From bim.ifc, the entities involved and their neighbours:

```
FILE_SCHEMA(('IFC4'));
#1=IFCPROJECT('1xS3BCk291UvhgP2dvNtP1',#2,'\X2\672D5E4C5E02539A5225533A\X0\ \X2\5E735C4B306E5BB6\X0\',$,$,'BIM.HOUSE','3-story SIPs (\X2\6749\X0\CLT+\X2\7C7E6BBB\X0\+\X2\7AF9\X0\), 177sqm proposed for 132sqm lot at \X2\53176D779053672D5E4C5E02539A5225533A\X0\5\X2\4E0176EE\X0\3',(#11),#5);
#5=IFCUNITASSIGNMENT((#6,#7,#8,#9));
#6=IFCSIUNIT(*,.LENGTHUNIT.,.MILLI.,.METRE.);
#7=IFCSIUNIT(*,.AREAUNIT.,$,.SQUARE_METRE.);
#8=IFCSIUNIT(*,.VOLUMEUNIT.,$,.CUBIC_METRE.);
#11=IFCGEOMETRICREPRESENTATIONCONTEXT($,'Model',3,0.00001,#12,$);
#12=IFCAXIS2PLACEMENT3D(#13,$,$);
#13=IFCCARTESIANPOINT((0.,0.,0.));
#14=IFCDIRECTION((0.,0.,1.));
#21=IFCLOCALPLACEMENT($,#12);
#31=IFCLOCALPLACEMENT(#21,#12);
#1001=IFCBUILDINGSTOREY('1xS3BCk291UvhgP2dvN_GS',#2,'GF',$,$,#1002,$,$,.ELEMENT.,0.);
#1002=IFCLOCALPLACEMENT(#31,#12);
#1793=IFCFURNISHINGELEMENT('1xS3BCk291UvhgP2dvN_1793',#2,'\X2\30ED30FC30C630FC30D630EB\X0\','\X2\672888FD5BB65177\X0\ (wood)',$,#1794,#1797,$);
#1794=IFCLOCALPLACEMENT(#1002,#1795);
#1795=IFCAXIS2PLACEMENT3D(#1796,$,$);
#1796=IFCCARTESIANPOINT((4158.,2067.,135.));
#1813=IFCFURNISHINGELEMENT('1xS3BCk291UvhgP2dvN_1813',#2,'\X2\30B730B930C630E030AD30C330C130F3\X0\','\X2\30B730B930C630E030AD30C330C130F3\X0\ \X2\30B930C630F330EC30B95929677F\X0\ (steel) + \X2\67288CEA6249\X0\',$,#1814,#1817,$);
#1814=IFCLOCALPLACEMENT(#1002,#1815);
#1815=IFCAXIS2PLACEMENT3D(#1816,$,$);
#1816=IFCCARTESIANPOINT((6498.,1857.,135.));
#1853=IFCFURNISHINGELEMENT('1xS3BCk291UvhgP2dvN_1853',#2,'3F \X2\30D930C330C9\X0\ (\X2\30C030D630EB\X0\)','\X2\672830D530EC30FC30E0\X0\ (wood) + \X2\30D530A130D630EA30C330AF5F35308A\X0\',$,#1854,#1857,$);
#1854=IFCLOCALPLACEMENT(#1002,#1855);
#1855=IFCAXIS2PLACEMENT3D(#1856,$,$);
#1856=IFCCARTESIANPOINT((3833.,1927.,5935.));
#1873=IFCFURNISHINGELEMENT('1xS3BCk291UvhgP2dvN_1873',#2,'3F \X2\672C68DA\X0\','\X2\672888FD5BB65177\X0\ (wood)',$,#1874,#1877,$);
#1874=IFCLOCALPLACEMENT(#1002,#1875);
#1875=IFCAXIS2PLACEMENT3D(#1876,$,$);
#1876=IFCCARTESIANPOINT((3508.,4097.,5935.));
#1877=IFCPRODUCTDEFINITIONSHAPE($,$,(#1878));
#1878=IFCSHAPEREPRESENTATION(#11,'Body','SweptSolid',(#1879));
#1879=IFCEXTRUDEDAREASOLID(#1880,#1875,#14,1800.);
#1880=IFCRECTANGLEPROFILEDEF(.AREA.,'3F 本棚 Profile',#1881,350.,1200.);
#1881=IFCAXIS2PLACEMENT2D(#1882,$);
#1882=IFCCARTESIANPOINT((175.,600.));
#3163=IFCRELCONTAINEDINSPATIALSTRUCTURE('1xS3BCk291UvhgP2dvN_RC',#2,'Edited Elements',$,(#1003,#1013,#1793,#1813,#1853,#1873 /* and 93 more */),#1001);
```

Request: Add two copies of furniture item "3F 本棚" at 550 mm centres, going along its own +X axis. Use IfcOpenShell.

```python
import ifcopenshell
import ifcopenshell.api.geometry
import ifcopenshell.api.root
import ifcopenshell.util.element
import ifcopenshell.util.placement
import ifcopenshell.util.unit

model = ifcopenshell.open("bim.ifc")
unit_scale = ifcopenshell.util.unit.calculate_unit_scale(model)


def reuse_history(source, copy):
    """copy_class also copies each property set's owner history, people and application; keep the originals."""
    for rel in copy.IsDefinedBy:
        if rel.is_a("IfcRelDefinesByProperties") and (history := rel.RelatingPropertyDefinition.OwnerHistory):
            rel.RelatingPropertyDefinition.OwnerHistory = source.OwnerHistory
            ifcopenshell.util.element.remove_deep2(model, history)


source = model.by_guid("1xS3BCk291UvhgP2dvN_1873")
base = ifcopenshell.util.placement.get_local_placement(source.ObjectPlacement)
step = base[:3, 0] * 0.55 / unit_scale

for i in range(1, 3):
    copy = ifcopenshell.api.root.copy_class(model, product=source)
    copy.Representation = ifcopenshell.util.element.copy_deep(
        model, source.Representation, exclude=["IfcGeometricRepresentationContext", "IfcRepresentationMap"]
    )
    reuse_history(source, copy)
    matrix = base.copy()
    matrix[:3, 3] += i * step
    print("added at", matrix[:3, 3].round(3) + 0.0)
    ifcopenshell.api.geometry.edit_object_placement(model, product=copy, matrix=matrix, is_si=False)

model.write("bim_v2.ifc")
```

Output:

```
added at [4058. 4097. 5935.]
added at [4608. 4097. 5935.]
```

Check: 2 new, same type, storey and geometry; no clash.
